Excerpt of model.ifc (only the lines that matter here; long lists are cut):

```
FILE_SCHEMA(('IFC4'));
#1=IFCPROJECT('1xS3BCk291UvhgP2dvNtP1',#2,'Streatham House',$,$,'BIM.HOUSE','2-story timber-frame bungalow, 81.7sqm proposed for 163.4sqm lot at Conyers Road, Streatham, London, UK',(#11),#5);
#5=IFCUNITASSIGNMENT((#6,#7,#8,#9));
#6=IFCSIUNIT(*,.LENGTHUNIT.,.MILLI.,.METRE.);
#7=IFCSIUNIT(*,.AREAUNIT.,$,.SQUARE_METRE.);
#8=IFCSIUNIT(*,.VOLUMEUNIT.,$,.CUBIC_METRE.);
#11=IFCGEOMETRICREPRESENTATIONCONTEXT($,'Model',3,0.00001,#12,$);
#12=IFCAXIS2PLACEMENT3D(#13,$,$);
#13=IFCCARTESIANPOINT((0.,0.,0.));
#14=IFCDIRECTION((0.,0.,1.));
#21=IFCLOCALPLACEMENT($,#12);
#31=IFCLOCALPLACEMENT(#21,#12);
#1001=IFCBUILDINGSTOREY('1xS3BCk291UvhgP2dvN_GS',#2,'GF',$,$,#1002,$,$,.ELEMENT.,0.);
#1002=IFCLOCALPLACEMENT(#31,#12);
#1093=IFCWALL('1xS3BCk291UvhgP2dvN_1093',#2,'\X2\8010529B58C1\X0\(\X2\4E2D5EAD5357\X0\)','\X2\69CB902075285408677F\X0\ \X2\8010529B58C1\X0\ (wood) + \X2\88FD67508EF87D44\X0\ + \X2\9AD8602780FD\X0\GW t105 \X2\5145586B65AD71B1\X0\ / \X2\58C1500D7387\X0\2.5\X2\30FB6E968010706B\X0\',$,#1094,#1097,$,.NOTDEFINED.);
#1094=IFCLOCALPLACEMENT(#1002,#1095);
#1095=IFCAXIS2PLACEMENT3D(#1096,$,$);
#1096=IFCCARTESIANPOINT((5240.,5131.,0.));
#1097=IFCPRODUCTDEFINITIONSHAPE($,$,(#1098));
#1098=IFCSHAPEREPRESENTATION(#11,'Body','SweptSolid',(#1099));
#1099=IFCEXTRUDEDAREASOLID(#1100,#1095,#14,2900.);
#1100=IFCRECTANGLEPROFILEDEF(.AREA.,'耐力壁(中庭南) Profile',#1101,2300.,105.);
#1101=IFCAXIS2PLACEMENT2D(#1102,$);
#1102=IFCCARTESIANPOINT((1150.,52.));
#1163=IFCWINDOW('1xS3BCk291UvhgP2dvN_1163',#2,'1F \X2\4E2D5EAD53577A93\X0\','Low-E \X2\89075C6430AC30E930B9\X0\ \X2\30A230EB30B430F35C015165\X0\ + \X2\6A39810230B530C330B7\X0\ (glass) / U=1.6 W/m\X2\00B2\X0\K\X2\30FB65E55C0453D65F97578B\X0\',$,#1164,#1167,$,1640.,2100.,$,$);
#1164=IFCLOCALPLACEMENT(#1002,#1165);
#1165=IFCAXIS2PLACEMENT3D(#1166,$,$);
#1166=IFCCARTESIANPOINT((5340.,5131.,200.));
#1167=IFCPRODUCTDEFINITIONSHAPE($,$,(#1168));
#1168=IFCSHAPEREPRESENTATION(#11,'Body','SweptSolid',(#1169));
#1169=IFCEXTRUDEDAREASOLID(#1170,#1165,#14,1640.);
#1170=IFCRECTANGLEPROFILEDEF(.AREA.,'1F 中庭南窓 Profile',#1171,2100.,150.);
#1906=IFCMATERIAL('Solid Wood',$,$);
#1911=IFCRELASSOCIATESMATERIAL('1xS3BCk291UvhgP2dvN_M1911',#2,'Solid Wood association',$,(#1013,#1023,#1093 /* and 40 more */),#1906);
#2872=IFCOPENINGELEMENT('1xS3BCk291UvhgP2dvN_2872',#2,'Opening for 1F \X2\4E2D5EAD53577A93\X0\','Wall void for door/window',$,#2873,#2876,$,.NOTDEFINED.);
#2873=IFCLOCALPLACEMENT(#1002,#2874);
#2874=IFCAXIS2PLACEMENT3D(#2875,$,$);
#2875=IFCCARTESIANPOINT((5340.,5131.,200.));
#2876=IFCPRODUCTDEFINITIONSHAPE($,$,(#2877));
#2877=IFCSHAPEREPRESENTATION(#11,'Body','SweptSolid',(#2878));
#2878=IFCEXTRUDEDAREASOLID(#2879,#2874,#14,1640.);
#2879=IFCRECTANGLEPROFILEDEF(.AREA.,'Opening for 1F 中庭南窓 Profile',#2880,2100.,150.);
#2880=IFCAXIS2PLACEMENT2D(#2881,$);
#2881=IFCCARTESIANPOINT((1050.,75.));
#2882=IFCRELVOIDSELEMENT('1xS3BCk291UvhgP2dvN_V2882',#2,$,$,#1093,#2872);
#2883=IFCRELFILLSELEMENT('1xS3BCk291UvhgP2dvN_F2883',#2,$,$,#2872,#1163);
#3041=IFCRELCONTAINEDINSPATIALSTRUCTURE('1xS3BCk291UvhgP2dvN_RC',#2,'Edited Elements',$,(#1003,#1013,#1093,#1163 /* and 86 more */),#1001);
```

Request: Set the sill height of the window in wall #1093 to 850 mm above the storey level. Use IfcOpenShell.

```python
import numpy as np
import ifcopenshell
import ifcopenshell.api.geometry
import ifcopenshell.geom
import ifcopenshell.util.element
import ifcopenshell.util.placement
import ifcopenshell.util.shape
import ifcopenshell.util.unit

model = ifcopenshell.open("model.ifc")
unit_scale = ifcopenshell.util.unit.calculate_unit_scale(model)

window = model.by_guid("1xS3BCk291UvhgP2dvN_1163")
opening = window.FillsVoids[0].RelatingOpeningElement
storey = ifcopenshell.util.element.get_container(window, ifc_class="IfcBuildingStorey")
level = ifcopenshell.util.placement.get_local_placement(storey.ObjectPlacement)[2, 3]

# The opening's origin need not be at the sill, so measure its lowest point.
shape = ifcopenshell.geom.create_shape(ifcopenshell.geom.settings(), opening)
bottom = ifcopenshell.util.shape.get_shape_bottom_elevation(shape, shape.geometry) / unit_scale
dz = level + 850.0 - bottom

shift = np.array([0.0, 0.0, dz])
# The window is not placed relative to its opening, so move both.
for product in (opening, window):
    matrix = ifcopenshell.util.placement.get_local_placement(product.ObjectPlacement)
    matrix[:3, 3] += shift
    ifcopenshell.api.geometry.edit_object_placement(model, product=product, matrix=matrix, is_si=False)

print(f"moved by {dz * unit_scale:+.3f} m")

model.write("model_edited.ifc")
```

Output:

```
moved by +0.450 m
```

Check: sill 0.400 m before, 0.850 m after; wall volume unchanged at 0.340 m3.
